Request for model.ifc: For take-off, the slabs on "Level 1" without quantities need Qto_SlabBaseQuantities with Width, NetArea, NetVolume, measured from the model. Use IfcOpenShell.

First a look at what the model holds.

```python
import ifcopenshell
import ifcopenshell.util.element
import ifcopenshell.util.unit

model = ifcopenshell.open("model.ifc")
print(model.schema)
for unit_type in ("LENGTHUNIT", "AREAUNIT", "VOLUMEUNIT"):
    print(unit_type, ifcopenshell.util.unit.calculate_unit_scale(model, unit_type))
storey = next(s for s in model.by_type("IfcBuildingStorey") if s.Name == "Level 1")
slabs = [e for e in ifcopenshell.util.element.get_decomposition(storey) if e.is_a("IfcSlab")]
for e in sorted(slabs, key=lambda e: e.id()):
    print(e.id(), e.is_a(), e.Name, list(ifcopenshell.util.element.get_psets(e, qtos_only=True)), sep=" | ")
```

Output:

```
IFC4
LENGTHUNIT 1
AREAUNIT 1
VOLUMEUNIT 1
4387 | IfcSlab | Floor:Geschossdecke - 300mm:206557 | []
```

```python
import ifcopenshell
import ifcopenshell.api.pset
import ifcopenshell.geom
import ifcopenshell.util.element
import ifcopenshell.util.shape
import ifcopenshell.util.unit

model = ifcopenshell.open("model.ifc")
unit_scale = ifcopenshell.util.unit.calculate_unit_scale(model)
area_scale = ifcopenshell.util.unit.calculate_unit_scale(model, "AREAUNIT")
volume_scale = ifcopenshell.util.unit.calculate_unit_scale(model, "VOLUMEUNIT")
settings = ifcopenshell.geom.settings()

storey = next(s for s in model.by_type("IfcBuildingStorey") if s.Name == "Level 1")
slabs = [e for e in ifcopenshell.util.element.get_decomposition(storey) if e.is_a("IfcSlab")]

for e in sorted(slabs, key=lambda e: e.id()):
    if ifcopenshell.util.element.get_psets(e, qtos_only=True, should_inherit=False):
        continue
    # Geometry comes back in metres, in the element's own axes.
    shape = ifcopenshell.geom.create_shape(settings, e)
    values = {
        "Width": ifcopenshell.util.shape.get_z(shape.geometry) / unit_scale,
        "NetArea": ifcopenshell.util.shape.get_footprint_area(shape.geometry) / area_scale,
        "NetVolume": ifcopenshell.util.shape.get_volume(shape.geometry) / volume_scale,
    }
    qto = ifcopenshell.api.pset.add_qto(model, product=e, name="Qto_SlabBaseQuantities")
    ifcopenshell.api.pset.edit_qto(model, qto=qto, properties=values)
    print(e.id(), {k: round(v, 3) for k, v in values.items()})

model.write("model_rev.ifc")
```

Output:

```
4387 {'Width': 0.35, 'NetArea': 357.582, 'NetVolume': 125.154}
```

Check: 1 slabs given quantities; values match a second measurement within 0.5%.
